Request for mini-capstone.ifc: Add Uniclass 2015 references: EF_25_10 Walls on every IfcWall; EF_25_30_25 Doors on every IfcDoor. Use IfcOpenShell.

First a look at what the model holds.

```python
import ifcopenshell

model = ifcopenshell.open("mini-capstone.ifc")
print(model.schema)
print("classifications:", [c.Name for c in model.by_type("IfcClassification")])
for ifc_class in ("IfcDoor", "IfcRoof", "IfcStair", "IfcWall", "IfcWindow"):
    print(ifc_class, len(model.by_type(ifc_class)))
```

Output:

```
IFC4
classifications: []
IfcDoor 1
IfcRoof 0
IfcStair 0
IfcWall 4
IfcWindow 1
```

```python
import ifcopenshell
import ifcopenshell.api.classification

model = ifcopenshell.open("mini-capstone.ifc")

system = ifcopenshell.api.classification.add_classification(model, classification="Uniclass 2015")

codes = {
    "IfcWall": ("EF_25_10", "Walls"),
    "IfcDoor": ("EF_25_30_25", "Doors"),
}
for ifc_class, (code, name) in codes.items():
    products = model.by_type(ifc_class)
    ifcopenshell.api.classification.add_reference(
        model, products=products, classification=system, identification=code, name=name
    )
    print(code, len(products))

model.write("mini-capstone_rev.ifc")
```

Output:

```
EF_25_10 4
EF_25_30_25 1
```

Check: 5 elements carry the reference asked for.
